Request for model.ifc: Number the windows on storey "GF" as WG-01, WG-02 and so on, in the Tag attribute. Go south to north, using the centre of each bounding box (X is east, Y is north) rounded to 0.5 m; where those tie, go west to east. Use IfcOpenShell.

First a look at what the model holds.

```python
import ifcopenshell
import ifcopenshell.util.element
import ifcopenshell.util.placement

model = ifcopenshell.open("model.ifc")
print(model.schema)
storey = next(s for s in model.by_type("IfcBuildingStorey") if s.Name == "GF")
windows = [e for e in ifcopenshell.util.element.get_decomposition(storey) if e.is_a("IfcWindow")]
for e in sorted(windows, key=lambda e: e.id()):
    origin = ifcopenshell.util.placement.get_local_placement(e.ObjectPlacement)[:3, 3]
    print(e.id(), e.Tag, e.Name, origin.round(2) + 0.0, sep=" | ")
```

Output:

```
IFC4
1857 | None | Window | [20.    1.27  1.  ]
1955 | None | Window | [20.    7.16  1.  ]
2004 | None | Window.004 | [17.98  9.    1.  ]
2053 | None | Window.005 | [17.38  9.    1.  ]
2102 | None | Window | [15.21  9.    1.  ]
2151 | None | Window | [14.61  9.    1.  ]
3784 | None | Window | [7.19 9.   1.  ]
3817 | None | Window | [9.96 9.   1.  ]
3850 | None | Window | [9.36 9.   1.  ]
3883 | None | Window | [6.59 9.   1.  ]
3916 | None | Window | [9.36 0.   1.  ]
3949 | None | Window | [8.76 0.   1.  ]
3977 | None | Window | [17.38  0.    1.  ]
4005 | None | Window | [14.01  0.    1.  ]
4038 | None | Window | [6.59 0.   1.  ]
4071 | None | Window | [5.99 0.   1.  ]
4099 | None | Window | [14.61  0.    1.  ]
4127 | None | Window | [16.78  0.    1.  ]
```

```python
import ifcopenshell
import ifcopenshell.geom
import ifcopenshell.util.element
import ifcopenshell.util.shape

model = ifcopenshell.open("model.ifc")
settings = ifcopenshell.geom.settings()
settings.set("use-world-coords", True)


def centre(element):
    shape = ifcopenshell.geom.create_shape(settings, element)
    return ifcopenshell.util.shape.get_bbox_centroid(shape.geometry)


storey = next(s for s in model.by_type("IfcBuildingStorey") if s.Name == "GF")
windows = [e for e in ifcopenshell.util.element.get_decomposition(storey) if e.is_a("IfcWindow")]

# Insertion points can sit at a corner or the storey origin, so sort by the geometry (in metres).
centres = {e: centre(e) for e in windows}
windows.sort(key=lambda e: (round(centres[e][1] / 0.5), centres[e][0]))

for i, e in enumerate(windows, start=1):
    number = f"WG-{i:02d}"
    e.Tag = number
    print(e.id(), number)

model.write("model-out.ifc")
```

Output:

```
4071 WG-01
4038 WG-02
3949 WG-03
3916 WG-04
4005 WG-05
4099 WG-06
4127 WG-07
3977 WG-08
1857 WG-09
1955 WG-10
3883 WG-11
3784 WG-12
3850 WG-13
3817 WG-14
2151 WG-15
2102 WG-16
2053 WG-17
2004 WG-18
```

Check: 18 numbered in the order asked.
